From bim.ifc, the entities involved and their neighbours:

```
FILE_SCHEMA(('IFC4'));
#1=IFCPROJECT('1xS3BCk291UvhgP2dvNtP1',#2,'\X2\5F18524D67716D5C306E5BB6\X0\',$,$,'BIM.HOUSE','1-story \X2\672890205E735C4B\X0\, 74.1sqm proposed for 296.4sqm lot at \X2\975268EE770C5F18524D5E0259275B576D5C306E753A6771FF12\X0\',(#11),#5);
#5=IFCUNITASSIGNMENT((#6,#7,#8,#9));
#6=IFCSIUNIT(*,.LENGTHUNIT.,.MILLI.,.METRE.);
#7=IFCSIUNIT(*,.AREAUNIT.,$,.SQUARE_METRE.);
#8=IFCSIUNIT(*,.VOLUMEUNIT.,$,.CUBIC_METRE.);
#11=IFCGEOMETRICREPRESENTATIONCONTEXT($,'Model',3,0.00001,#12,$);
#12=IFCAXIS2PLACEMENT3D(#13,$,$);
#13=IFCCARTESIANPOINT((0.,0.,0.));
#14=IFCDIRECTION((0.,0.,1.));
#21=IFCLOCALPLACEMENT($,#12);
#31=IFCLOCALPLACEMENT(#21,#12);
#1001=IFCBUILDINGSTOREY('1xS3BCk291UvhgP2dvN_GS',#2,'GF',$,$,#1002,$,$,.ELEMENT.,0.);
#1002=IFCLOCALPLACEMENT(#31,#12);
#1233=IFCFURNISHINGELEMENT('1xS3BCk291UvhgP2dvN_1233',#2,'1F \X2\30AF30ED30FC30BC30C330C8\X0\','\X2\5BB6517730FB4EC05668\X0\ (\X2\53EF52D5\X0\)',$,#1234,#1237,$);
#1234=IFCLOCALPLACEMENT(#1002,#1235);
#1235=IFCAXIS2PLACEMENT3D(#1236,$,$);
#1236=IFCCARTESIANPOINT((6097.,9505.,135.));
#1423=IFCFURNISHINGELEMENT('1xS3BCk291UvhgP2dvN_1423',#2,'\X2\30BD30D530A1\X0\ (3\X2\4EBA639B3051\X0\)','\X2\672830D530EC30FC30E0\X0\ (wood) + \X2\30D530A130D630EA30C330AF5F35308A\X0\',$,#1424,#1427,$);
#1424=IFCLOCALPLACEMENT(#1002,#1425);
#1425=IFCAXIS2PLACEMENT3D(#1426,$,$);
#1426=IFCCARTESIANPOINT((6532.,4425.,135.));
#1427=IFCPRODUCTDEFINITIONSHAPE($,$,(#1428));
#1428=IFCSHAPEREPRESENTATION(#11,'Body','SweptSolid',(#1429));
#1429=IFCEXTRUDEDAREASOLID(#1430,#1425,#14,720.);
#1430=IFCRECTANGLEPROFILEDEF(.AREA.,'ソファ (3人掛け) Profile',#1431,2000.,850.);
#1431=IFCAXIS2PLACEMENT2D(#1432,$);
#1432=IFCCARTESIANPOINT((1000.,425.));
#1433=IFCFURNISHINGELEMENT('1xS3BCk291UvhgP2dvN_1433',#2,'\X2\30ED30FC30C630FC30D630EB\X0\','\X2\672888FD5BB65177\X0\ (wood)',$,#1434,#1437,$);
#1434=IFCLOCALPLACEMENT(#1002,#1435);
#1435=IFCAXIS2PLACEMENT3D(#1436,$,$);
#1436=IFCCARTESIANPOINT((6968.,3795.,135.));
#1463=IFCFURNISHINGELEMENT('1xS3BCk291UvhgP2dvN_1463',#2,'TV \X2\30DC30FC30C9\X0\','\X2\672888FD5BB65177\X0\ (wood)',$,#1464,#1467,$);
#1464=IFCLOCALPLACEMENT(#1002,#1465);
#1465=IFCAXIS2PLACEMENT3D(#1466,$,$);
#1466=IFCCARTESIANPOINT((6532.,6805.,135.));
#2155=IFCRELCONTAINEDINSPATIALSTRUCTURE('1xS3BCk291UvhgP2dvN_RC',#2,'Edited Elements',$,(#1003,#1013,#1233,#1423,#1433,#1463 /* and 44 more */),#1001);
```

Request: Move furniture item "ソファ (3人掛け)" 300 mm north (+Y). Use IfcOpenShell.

```python
import ifcopenshell
import ifcopenshell.api.geometry
import ifcopenshell.util.placement
import ifcopenshell.util.unit

model = ifcopenshell.open("bim.ifc")
unit_scale = ifcopenshell.util.unit.calculate_unit_scale(model)

item = model.by_guid("1xS3BCk291UvhgP2dvN_1423")
matrix = ifcopenshell.util.placement.get_local_placement(item.ObjectPlacement)
matrix[1, 3] += 0.3 / unit_scale
ifcopenshell.api.geometry.edit_object_placement(model, product=item, matrix=matrix, is_si=False)

print(ifcopenshell.util.placement.get_local_placement(item.ObjectPlacement).round(3) + 0.0)

model.write("bim_rev.ifc")
```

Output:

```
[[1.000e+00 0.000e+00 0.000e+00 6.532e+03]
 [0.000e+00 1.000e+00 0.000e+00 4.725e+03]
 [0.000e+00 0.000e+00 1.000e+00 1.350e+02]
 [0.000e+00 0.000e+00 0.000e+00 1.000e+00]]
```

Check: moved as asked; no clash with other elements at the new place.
